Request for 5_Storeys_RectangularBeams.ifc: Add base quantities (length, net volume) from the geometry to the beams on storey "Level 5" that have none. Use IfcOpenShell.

First a look at what the model holds.

```python
import ifcopenshell
import ifcopenshell.util.element
import ifcopenshell.util.unit

model = ifcopenshell.open("5_Storeys_RectangularBeams.ifc")
print(model.schema)
for unit_type in ("LENGTHUNIT", "AREAUNIT", "VOLUMEUNIT"):
    print(unit_type, ifcopenshell.util.unit.calculate_unit_scale(model, unit_type))
storey = next(s for s in model.by_type("IfcBuildingStorey") if s.Name == "Level 5")
beams = [e for e in ifcopenshell.util.element.get_decomposition(storey) if e.is_a("IfcBeam")]
for e in sorted(beams, key=lambda e: e.id()):
    print(e.id(), e.is_a(), e.Name, list(ifcopenshell.util.element.get_psets(e, qtos_only=True)), sep=" | ")
```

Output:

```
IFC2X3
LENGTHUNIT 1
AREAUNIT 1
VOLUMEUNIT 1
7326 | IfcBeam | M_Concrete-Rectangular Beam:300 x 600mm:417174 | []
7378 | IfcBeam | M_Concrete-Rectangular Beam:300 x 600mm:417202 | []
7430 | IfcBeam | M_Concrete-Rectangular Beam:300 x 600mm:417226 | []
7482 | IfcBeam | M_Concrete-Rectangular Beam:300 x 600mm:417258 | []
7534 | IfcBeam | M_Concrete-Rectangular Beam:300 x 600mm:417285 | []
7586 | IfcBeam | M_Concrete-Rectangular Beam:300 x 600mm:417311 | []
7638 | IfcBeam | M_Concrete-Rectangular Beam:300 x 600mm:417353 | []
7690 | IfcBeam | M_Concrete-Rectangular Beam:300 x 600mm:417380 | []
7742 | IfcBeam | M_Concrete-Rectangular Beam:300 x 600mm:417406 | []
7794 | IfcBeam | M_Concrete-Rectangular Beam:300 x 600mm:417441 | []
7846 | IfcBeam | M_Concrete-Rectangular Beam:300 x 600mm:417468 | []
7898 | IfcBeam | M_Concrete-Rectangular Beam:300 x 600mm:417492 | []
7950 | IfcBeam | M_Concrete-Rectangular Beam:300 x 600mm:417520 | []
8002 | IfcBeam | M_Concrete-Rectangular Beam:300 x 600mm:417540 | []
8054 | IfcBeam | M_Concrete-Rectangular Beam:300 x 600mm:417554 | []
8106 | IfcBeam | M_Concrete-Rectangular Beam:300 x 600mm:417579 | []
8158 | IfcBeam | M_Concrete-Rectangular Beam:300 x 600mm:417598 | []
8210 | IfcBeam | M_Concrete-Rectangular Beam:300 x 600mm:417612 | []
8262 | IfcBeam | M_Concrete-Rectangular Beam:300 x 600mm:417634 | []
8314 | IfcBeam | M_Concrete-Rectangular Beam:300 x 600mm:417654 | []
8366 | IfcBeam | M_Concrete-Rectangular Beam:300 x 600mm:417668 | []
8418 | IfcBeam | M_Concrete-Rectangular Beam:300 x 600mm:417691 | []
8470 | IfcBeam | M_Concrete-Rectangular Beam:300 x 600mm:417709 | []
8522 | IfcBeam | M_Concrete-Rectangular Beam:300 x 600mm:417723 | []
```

```python
import ifcopenshell
import ifcopenshell.api.pset
import ifcopenshell.geom
import ifcopenshell.util.element
import ifcopenshell.util.shape
import ifcopenshell.util.unit

model = ifcopenshell.open("5_Storeys_RectangularBeams.ifc")
unit_scale = ifcopenshell.util.unit.calculate_unit_scale(model)
volume_scale = ifcopenshell.util.unit.calculate_unit_scale(model, "VOLUMEUNIT")
settings = ifcopenshell.geom.settings()

storey = next(s for s in model.by_type("IfcBuildingStorey") if s.Name == "Level 5")
beams = [e for e in ifcopenshell.util.element.get_decomposition(storey) if e.is_a("IfcBeam")]

for e in sorted(beams, key=lambda e: e.id()):
    if ifcopenshell.util.element.get_psets(e, qtos_only=True, should_inherit=False):
        continue
    # Geometry comes back in metres, in the element's own axes.
    shape = ifcopenshell.geom.create_shape(settings, e)
    values = {
        "Length": ifcopenshell.util.shape.get_max_xyz(shape.geometry) / unit_scale,
        "NetVolume": ifcopenshell.util.shape.get_volume(shape.geometry) / volume_scale,
    }
    qto = ifcopenshell.api.pset.add_qto(model, product=e, name="BaseQuantities")
    ifcopenshell.api.pset.edit_qto(model, qto=qto, properties=values)
    print(e.id(), {k: round(v, 3) for k, v in values.items()})

model.write("5_Storeys_RectangularBeams_edited.ifc")
```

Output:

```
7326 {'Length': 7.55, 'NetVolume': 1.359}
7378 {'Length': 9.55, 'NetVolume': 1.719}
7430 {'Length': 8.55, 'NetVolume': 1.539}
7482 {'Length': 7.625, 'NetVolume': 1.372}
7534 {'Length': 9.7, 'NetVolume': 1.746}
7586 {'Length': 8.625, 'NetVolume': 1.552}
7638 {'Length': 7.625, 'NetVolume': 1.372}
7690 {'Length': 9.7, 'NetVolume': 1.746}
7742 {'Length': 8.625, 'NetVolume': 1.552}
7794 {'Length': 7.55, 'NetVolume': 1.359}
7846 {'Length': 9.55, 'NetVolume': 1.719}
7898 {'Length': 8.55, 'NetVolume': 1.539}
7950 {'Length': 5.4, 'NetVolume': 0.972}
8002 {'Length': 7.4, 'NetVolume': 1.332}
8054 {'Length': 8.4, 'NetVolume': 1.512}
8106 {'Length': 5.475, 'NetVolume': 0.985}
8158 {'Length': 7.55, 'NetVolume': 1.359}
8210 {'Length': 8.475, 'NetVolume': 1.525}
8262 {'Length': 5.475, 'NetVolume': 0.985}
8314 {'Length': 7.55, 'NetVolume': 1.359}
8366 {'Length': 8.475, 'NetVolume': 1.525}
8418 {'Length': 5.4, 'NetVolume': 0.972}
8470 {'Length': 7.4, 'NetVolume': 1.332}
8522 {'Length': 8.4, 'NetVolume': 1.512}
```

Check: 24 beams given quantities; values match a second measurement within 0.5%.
